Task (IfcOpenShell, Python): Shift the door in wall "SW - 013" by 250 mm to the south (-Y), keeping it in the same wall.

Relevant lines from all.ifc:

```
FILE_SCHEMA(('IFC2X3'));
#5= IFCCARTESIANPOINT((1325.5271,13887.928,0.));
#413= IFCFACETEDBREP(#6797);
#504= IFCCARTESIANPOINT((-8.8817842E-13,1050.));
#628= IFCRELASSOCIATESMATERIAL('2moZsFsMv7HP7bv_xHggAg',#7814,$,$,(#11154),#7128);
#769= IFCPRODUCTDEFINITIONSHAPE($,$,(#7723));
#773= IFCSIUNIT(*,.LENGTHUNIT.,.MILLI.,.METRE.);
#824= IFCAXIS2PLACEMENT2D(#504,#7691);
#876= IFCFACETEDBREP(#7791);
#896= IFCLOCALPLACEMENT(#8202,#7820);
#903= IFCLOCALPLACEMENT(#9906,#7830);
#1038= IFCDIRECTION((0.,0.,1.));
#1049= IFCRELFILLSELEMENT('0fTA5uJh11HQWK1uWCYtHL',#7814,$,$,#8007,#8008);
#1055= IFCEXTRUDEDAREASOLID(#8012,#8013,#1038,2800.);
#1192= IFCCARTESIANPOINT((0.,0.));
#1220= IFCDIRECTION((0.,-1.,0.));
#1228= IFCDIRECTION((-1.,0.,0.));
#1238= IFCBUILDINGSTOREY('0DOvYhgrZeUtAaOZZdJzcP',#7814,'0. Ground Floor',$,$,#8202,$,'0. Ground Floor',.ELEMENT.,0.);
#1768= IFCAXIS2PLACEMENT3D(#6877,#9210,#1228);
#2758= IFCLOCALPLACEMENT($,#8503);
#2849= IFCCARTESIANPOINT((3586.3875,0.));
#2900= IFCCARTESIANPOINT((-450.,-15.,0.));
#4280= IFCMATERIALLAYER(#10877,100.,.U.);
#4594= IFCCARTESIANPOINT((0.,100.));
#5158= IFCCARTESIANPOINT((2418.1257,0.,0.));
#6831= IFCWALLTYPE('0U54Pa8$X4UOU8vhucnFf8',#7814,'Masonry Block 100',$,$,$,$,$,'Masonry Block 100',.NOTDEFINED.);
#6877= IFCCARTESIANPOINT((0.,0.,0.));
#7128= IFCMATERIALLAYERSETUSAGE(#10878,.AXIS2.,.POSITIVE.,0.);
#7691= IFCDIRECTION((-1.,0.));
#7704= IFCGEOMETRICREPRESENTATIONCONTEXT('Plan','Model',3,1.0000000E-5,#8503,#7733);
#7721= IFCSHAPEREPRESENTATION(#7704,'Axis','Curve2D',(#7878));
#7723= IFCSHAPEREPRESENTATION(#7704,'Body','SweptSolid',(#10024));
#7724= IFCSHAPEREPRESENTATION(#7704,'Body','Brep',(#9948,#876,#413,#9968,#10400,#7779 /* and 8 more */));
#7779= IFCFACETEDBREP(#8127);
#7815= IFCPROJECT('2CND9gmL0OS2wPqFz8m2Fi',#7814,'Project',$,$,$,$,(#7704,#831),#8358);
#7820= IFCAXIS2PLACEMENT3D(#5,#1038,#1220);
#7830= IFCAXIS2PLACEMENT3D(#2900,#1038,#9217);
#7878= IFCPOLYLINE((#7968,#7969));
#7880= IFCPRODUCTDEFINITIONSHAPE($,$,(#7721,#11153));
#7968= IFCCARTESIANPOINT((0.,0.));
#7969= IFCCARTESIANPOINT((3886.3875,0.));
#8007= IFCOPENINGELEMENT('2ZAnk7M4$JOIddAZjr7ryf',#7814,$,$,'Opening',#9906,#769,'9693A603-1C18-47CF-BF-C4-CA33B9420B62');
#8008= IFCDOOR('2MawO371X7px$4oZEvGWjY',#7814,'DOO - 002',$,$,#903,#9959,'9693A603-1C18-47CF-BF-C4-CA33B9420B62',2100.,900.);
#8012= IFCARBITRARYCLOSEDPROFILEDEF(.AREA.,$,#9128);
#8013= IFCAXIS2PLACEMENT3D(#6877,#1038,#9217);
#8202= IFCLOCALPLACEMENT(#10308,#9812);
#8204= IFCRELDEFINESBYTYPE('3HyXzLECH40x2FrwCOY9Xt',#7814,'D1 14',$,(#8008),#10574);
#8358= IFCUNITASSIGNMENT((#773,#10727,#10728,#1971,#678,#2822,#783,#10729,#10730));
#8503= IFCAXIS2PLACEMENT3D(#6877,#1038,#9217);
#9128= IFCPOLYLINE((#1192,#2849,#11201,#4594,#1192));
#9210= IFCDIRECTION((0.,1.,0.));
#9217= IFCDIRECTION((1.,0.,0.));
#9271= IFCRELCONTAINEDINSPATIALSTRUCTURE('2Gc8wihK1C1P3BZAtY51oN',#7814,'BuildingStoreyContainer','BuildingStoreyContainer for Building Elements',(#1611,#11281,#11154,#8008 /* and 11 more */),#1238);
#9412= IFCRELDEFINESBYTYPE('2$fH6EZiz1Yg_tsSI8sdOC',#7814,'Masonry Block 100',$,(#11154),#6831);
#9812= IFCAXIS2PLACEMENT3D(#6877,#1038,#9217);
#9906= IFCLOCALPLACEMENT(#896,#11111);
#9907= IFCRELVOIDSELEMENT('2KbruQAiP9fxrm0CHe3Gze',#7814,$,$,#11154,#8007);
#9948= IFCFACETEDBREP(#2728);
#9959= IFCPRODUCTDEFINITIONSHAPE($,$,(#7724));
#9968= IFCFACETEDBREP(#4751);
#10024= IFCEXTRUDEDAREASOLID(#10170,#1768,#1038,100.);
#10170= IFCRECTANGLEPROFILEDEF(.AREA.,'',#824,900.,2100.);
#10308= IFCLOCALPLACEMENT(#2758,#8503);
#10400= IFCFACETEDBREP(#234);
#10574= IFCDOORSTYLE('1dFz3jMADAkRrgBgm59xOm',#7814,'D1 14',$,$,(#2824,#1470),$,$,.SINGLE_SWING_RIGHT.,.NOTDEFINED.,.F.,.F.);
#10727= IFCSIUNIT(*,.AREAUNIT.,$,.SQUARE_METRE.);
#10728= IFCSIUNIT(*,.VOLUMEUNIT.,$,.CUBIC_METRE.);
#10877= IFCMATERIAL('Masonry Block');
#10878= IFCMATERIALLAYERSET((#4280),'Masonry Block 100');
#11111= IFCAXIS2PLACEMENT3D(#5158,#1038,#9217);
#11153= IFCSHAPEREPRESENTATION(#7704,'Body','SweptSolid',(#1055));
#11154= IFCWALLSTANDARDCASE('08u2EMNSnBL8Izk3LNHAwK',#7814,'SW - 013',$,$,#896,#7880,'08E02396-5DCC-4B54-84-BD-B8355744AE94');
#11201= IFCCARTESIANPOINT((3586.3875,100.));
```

```python
import ifcopenshell
import ifcopenshell.api.geometry
import ifcopenshell.util.placement
import ifcopenshell.util.unit

model = ifcopenshell.open("all.ifc")
unit_scale = ifcopenshell.util.unit.calculate_unit_scale(model)

door = model.by_guid("2MawO371X7px$4oZEvGWjY")
opening = door.FillsVoids[0].RelatingOpeningElement
wall = opening.VoidsElements[0].RelatingBuildingElement

wall_matrix = ifcopenshell.util.placement.get_local_placement(wall.ObjectPlacement)
shift = wall_matrix[:3, 0] * 0.25 / unit_scale
before = ifcopenshell.util.placement.get_local_placement(door.ObjectPlacement)[:3, 3].copy()

# The door is placed relative to its opening, so it follows when the opening moves.
matrix = ifcopenshell.util.placement.get_local_placement(opening.ObjectPlacement)
matrix[:3, 3] += shift
ifcopenshell.api.geometry.edit_object_placement(
    model, product=opening, matrix=matrix, is_si=False, should_transform_children=True
)

after = ifcopenshell.util.placement.get_local_placement(door.ObjectPlacement)[:3, 3]
print("door moved by", (after - before).round(3) + 0.0)

model.write("all_rev.ifc")
```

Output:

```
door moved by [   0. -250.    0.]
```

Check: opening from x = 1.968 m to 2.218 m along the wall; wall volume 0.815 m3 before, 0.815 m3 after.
